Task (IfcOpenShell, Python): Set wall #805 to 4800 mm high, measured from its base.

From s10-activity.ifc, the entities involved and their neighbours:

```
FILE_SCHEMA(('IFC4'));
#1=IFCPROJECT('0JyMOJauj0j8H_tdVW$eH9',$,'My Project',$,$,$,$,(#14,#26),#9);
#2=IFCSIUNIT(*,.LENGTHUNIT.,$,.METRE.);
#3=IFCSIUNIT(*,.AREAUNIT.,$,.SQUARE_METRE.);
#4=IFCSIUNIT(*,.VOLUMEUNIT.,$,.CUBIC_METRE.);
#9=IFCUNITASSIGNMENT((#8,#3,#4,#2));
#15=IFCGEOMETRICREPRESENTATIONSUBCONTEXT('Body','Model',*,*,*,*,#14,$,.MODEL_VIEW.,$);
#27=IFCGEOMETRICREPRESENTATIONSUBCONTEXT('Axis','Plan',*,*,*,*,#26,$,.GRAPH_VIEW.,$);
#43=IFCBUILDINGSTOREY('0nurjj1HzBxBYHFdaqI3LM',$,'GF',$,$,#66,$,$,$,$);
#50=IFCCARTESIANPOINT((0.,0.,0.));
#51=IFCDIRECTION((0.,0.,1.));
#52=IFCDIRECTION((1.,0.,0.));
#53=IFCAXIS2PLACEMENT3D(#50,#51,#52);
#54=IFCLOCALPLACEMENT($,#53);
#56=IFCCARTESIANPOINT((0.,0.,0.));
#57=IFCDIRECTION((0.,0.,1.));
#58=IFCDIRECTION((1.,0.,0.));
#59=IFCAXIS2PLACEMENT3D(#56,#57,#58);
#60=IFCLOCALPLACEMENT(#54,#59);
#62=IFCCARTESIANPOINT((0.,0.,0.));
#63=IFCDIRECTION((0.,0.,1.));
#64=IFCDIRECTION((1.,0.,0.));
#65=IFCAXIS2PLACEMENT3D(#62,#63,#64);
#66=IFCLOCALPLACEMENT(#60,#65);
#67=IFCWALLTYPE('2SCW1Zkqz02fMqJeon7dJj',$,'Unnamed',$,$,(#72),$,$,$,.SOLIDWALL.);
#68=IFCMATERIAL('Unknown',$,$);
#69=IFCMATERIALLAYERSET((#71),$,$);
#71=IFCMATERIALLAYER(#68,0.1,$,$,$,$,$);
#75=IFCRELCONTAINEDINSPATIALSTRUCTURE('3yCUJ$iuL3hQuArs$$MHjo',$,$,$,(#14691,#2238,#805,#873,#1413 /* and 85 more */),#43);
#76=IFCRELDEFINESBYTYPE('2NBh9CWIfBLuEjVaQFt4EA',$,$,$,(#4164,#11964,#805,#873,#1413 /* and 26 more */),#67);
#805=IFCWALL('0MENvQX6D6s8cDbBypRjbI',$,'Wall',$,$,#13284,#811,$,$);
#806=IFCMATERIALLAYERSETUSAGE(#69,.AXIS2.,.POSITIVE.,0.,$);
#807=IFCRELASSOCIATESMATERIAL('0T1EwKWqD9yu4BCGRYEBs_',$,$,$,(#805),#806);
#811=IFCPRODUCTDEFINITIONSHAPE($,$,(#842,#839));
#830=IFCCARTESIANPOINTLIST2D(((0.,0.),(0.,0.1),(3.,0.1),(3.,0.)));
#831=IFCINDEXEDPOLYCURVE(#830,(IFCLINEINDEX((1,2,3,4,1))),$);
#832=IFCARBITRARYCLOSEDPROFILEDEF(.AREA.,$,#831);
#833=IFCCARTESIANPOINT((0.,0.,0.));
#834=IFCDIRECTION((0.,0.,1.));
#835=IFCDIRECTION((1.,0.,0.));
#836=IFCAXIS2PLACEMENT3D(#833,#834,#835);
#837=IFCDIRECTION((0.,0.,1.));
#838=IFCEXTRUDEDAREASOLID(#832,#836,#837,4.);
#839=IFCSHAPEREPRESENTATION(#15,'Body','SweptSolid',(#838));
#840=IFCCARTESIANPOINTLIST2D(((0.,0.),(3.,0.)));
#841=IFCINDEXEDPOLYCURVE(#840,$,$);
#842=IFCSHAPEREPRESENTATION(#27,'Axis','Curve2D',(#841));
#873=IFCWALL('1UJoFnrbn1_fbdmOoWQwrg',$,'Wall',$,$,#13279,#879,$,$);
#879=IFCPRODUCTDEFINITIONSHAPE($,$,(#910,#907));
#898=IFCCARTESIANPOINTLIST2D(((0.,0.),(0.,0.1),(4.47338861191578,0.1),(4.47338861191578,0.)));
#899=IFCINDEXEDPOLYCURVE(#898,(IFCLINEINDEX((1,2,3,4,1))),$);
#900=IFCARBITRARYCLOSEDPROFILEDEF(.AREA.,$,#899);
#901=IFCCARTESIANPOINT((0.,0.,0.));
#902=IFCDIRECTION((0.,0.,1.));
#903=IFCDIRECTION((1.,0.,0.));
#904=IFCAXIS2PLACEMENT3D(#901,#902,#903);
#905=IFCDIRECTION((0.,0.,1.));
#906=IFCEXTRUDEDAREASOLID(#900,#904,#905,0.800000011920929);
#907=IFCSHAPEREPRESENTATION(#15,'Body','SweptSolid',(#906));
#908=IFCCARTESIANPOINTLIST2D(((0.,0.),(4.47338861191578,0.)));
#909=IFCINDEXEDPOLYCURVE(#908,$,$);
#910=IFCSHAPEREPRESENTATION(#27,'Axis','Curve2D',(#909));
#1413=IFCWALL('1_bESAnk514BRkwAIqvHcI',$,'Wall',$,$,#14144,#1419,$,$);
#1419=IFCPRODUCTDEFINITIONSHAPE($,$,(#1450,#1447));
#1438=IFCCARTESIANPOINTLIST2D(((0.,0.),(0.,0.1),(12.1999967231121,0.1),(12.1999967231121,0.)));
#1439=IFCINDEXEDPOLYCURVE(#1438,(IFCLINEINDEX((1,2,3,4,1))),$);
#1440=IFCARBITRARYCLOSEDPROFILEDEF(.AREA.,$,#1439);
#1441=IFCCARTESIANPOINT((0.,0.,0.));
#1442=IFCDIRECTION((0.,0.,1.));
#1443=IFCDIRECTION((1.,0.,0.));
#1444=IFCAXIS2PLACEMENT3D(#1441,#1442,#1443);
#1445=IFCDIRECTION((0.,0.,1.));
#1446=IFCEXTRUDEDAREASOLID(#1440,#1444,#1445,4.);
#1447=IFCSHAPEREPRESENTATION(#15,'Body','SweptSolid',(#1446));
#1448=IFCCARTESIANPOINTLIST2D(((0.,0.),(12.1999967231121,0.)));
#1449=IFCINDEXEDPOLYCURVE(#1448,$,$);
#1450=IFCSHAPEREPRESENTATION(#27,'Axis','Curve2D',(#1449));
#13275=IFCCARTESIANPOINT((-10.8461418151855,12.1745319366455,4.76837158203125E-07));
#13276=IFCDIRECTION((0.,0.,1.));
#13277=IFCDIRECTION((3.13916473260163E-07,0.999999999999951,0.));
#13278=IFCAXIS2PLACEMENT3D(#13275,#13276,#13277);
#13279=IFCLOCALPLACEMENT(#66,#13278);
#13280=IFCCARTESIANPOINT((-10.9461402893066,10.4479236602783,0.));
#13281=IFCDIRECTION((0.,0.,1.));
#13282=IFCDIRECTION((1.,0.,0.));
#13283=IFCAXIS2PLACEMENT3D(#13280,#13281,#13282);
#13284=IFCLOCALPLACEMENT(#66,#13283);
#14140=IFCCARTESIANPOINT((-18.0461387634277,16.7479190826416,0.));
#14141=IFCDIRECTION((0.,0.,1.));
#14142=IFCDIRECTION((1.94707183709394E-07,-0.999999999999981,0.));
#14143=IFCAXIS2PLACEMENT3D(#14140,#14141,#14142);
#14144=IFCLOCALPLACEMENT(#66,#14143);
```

```python
import ifcopenshell
import ifcopenshell.geom
import ifcopenshell.util.representation
import ifcopenshell.util.shape
import ifcopenshell.util.unit

model = ifcopenshell.open("s10-activity.ifc")
unit_scale = ifcopenshell.util.unit.calculate_unit_scale(model)
settings = ifcopenshell.geom.settings()


def volume(element):
    """Net volume in cubic metres, openings subtracted."""
    shape = ifcopenshell.geom.create_shape(settings, element)
    return ifcopenshell.util.shape.get_volume(shape.geometry)


wall = model.by_id(805)
before = volume(wall)

body = ifcopenshell.util.representation.get_representation(wall, "Model", "Body")
solid = body.Items[0]
old_height = solid.Depth
solid.Depth = 4.8 / unit_scale
after = volume(wall)

print(f"height {old_height:g} -> {solid.Depth:g}, volume {before:.3f} -> {after:.3f} m3")

model.write("s10-activity_edited.ifc")
```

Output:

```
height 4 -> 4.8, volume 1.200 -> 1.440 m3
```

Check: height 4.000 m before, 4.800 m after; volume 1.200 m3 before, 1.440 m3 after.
